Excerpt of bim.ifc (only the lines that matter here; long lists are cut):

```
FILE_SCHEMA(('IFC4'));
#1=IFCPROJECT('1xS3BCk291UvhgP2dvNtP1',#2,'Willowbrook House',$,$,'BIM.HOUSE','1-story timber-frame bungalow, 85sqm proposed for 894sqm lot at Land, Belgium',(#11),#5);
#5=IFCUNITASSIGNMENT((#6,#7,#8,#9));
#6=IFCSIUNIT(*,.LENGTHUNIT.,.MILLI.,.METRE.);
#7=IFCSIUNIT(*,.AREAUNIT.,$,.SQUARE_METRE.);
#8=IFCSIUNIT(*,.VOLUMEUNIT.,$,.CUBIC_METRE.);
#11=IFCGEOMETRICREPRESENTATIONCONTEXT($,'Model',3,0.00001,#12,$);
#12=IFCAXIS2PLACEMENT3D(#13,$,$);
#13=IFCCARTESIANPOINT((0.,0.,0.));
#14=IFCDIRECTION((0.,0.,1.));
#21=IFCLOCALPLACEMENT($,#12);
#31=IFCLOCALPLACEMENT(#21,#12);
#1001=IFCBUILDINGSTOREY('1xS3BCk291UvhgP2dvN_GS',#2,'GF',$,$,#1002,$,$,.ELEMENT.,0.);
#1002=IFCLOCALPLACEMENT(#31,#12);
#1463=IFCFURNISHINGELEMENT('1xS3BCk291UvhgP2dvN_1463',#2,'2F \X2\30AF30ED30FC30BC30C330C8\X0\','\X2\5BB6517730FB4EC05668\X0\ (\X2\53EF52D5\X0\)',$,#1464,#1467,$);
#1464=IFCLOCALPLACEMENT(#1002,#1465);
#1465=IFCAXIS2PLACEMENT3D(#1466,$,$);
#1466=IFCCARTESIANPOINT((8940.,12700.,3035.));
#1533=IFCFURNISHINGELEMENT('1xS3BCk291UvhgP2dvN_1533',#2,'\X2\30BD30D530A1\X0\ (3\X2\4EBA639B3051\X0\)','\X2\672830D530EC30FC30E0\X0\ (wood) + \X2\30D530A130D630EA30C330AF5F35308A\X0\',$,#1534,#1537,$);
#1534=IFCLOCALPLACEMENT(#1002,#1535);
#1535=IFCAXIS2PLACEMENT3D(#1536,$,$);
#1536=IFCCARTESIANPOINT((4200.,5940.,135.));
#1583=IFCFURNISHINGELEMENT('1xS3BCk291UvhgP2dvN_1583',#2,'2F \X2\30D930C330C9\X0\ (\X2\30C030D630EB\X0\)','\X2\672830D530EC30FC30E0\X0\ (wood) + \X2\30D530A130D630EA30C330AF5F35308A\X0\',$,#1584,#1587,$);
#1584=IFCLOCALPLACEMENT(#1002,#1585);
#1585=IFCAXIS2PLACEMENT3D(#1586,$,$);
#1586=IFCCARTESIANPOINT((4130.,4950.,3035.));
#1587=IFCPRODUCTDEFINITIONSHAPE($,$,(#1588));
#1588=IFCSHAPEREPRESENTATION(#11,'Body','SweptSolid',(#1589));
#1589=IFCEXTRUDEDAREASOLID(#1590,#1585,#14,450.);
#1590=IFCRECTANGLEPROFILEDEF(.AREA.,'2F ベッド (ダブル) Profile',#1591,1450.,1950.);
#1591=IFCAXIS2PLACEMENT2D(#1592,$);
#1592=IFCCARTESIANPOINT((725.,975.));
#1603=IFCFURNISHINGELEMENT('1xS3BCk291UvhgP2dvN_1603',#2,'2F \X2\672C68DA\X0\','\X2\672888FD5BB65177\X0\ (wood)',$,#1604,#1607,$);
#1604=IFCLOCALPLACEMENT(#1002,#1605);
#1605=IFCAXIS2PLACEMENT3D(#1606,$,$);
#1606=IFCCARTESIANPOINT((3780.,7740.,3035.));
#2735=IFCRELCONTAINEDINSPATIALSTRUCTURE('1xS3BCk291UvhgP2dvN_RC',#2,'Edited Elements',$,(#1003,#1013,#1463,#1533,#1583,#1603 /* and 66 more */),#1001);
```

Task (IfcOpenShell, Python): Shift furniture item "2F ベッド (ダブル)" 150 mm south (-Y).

```python
import ifcopenshell
import ifcopenshell.api.geometry
import ifcopenshell.util.placement

model = ifcopenshell.open("bim.ifc")

item = model.by_guid("1xS3BCk291UvhgP2dvN_1583")
matrix = ifcopenshell.util.placement.get_local_placement(item.ObjectPlacement)
matrix[1, 3] -= 150.0
ifcopenshell.api.geometry.edit_object_placement(model, product=item, matrix=matrix, is_si=False)

print(ifcopenshell.util.placement.get_local_placement(item.ObjectPlacement).round(3) + 0.0)

model.write("bim-out.ifc")
```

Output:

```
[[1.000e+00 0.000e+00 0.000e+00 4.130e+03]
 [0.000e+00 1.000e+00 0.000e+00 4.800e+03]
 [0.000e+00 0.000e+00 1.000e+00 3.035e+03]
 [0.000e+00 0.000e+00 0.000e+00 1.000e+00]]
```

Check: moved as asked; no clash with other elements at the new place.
